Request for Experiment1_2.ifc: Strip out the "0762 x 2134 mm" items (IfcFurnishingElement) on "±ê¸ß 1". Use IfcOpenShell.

First a look at what the model holds.

```python
import ifcopenshell
import ifcopenshell.util.element

model = ifcopenshell.open("Experiment1_2.ifc")
print(model.schema)
storey = next(s for s in model.by_type("IfcBuildingStorey") if s.Name == "±ê¸ß 1")
furniture = [e for e in ifcopenshell.util.element.get_decomposition(storey) if e.is_a("IfcFurnishingElement")]
seen = {}
for e in furniture:
    element_type = ifcopenshell.util.element.get_type(e)
    name = element_type.Name if element_type not in (None, e) else None
    seen[name] = seen.get(name, 0) + 1
for name, count in sorted(seen.items(), key=str):
    print(count, "x", name)
```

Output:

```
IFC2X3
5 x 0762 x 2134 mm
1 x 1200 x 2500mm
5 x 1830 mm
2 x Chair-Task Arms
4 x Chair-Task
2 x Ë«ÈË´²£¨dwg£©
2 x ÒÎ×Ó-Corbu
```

```python
import ifcopenshell
import ifcopenshell.api.root
import ifcopenshell.util.element

model = ifcopenshell.open("Experiment1_2.ifc")

storey = next(s for s in model.by_type("IfcBuildingStorey") if s.Name == "±ê¸ß 1")
furniture = [e for e in ifcopenshell.util.element.get_decomposition(storey) if e.is_a("IfcFurnishingElement")]
targets = [e for e in furniture if (t := ifcopenshell.util.element.get_type(e)) not in (None, e) and t.Name == "0762 x 2134 mm"]

for e in targets:
    ifcopenshell.api.root.remove_product(model, product=e)
print(len(targets), "removed")

model.write("Experiment1_2_rev.ifc")
```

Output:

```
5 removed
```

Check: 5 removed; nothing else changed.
